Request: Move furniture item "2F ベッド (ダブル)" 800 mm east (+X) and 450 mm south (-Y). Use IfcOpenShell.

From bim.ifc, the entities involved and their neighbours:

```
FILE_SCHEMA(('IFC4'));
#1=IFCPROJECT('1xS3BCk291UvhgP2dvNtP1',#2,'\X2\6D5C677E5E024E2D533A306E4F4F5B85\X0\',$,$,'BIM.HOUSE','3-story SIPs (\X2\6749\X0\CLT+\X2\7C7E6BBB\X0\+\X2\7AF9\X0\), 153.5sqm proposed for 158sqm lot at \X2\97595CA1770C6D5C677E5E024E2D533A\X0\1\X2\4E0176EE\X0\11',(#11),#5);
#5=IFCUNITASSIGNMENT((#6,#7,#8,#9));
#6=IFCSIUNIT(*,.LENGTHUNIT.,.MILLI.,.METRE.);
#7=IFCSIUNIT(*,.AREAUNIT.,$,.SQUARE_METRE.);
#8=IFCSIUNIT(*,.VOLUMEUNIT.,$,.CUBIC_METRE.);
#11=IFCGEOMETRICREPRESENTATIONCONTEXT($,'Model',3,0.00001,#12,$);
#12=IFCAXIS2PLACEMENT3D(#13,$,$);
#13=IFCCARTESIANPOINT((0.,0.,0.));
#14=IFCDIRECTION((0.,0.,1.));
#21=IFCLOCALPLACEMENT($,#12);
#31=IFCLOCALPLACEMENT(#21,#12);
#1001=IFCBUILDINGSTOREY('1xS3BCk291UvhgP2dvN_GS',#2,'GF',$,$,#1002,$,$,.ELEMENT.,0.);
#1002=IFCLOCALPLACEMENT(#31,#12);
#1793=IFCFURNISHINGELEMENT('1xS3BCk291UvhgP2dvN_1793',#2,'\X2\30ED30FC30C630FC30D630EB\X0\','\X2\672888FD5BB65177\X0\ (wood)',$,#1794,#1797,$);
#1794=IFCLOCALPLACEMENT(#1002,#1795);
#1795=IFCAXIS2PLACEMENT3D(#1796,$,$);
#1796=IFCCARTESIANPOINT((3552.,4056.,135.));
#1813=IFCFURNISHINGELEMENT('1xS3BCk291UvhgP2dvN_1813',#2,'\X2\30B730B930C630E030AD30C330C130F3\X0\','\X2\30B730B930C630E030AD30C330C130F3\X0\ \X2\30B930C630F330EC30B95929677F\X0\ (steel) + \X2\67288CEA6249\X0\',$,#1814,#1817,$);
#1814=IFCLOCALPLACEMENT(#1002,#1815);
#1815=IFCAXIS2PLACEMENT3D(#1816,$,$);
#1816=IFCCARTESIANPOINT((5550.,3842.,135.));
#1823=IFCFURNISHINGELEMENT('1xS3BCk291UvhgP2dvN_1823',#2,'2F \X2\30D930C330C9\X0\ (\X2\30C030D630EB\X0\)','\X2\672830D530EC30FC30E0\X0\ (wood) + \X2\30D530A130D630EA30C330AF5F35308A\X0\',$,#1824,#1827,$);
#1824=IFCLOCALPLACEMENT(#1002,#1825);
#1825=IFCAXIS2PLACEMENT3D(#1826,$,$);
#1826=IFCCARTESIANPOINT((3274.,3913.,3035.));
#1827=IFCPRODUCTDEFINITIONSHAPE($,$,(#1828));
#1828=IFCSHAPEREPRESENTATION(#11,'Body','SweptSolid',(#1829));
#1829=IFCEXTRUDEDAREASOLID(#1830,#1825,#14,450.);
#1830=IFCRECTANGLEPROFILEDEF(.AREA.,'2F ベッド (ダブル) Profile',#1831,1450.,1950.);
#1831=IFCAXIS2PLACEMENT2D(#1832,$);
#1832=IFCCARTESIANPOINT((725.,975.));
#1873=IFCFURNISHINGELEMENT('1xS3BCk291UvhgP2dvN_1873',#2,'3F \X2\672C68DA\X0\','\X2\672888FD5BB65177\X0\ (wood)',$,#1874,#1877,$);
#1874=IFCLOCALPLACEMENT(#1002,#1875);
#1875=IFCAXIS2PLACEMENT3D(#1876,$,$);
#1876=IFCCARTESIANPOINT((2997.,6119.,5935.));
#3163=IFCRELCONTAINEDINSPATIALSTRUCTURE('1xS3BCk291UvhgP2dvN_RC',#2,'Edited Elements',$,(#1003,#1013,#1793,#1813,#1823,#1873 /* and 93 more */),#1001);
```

```python
import ifcopenshell
import ifcopenshell.api.geometry
import ifcopenshell.util.placement

model = ifcopenshell.open("bim.ifc")

item = model.by_id(1823)
matrix = ifcopenshell.util.placement.get_local_placement(item.ObjectPlacement)
matrix[0, 3] += 800.0
matrix[1, 3] -= 450.0
ifcopenshell.api.geometry.edit_object_placement(model, product=item, matrix=matrix, is_si=False)

print(ifcopenshell.util.placement.get_local_placement(item.ObjectPlacement).round(3) + 0.0)

model.write("bim_edited.ifc")
```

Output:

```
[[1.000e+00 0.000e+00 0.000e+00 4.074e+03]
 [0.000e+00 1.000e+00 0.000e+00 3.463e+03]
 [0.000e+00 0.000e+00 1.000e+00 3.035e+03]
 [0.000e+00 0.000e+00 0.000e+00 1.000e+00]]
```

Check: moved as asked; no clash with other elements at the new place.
